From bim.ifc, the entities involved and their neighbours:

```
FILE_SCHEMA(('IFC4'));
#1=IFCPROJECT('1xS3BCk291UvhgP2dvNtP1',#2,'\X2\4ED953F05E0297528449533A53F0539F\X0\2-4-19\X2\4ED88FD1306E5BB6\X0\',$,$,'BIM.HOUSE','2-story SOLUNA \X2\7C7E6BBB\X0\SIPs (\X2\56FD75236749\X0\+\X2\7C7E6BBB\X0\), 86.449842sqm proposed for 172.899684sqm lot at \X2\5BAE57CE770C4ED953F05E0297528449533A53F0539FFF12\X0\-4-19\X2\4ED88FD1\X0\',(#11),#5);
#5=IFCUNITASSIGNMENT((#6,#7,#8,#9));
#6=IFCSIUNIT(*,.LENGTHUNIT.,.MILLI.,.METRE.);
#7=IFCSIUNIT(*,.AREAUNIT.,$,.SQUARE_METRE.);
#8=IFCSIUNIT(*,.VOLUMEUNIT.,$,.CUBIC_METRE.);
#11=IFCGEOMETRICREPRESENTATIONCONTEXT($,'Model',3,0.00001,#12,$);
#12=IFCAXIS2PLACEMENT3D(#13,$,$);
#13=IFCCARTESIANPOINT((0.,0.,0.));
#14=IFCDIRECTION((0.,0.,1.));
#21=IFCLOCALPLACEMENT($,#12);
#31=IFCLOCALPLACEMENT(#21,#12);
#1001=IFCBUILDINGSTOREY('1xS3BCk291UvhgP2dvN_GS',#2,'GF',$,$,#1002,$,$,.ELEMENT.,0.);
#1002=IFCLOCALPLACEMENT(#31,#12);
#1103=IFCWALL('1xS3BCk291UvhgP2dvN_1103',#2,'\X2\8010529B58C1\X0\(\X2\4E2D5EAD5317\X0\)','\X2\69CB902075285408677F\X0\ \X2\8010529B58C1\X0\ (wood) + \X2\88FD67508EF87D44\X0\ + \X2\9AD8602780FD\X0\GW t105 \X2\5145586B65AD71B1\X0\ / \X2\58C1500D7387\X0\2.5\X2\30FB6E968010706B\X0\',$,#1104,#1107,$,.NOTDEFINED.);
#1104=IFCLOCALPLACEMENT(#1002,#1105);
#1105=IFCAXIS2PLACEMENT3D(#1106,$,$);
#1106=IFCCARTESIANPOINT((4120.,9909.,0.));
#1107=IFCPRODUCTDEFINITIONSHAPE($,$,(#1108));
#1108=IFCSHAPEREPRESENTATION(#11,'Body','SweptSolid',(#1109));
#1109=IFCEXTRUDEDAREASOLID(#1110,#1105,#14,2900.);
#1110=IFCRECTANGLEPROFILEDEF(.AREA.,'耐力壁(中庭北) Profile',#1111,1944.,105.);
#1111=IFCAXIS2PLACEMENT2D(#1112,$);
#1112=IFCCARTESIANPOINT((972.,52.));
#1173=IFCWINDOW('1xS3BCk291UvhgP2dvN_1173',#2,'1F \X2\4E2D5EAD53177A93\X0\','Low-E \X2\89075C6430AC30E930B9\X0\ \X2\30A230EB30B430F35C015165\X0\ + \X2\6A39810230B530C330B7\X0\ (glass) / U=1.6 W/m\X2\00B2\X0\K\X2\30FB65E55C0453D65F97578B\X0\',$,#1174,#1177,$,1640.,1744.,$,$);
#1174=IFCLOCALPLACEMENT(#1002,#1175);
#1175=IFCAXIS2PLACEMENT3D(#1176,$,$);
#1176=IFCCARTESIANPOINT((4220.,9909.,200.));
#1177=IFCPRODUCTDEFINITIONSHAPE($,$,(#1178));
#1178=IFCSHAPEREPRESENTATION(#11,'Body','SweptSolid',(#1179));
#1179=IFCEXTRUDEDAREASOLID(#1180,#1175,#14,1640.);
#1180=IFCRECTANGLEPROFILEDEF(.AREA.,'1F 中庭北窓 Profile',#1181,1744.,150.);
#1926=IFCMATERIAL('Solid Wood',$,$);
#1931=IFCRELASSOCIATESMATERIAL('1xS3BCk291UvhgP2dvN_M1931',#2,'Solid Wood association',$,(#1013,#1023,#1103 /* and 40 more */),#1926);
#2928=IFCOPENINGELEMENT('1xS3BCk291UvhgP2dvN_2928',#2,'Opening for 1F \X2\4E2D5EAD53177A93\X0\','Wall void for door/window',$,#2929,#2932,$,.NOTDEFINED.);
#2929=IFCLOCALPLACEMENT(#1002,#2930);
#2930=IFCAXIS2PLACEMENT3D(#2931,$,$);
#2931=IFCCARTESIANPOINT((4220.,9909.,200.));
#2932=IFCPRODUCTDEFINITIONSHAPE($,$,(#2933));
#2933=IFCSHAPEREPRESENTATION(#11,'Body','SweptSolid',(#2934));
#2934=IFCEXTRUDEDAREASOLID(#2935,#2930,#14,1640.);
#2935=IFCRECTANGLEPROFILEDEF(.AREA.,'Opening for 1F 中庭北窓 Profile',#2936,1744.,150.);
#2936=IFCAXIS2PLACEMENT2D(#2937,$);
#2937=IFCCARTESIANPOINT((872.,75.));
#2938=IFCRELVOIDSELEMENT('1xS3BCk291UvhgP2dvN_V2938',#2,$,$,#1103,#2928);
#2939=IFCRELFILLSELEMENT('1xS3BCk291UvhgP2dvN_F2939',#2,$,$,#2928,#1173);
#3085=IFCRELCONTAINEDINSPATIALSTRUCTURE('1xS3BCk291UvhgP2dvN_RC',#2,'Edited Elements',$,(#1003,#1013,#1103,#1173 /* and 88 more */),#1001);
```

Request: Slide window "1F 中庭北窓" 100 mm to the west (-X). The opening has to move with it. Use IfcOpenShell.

```python
import ifcopenshell
import ifcopenshell.api.geometry
import ifcopenshell.util.placement
import ifcopenshell.util.unit

model = ifcopenshell.open("bim.ifc")
unit_scale = ifcopenshell.util.unit.calculate_unit_scale(model)

window = model.by_guid("1xS3BCk291UvhgP2dvN_1173")
opening = window.FillsVoids[0].RelatingOpeningElement
wall = opening.VoidsElements[0].RelatingBuildingElement

wall_matrix = ifcopenshell.util.placement.get_local_placement(wall.ObjectPlacement)
shift = wall_matrix[:3, 0] * -0.1 / unit_scale
before = ifcopenshell.util.placement.get_local_placement(window.ObjectPlacement)[:3, 3].copy()

# The window is not placed relative to its opening, so move both.
for product in (opening, window):
    matrix = ifcopenshell.util.placement.get_local_placement(product.ObjectPlacement)
    matrix[:3, 3] += shift
    ifcopenshell.api.geometry.edit_object_placement(model, product=product, matrix=matrix, is_si=False)

after = ifcopenshell.util.placement.get_local_placement(window.ObjectPlacement)[:3, 3]
print("window moved by", (after - before).round(3) + 0.0)

model.write("bim_rev.ifc")
```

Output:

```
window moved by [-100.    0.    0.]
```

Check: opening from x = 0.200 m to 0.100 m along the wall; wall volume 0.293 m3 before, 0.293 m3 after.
